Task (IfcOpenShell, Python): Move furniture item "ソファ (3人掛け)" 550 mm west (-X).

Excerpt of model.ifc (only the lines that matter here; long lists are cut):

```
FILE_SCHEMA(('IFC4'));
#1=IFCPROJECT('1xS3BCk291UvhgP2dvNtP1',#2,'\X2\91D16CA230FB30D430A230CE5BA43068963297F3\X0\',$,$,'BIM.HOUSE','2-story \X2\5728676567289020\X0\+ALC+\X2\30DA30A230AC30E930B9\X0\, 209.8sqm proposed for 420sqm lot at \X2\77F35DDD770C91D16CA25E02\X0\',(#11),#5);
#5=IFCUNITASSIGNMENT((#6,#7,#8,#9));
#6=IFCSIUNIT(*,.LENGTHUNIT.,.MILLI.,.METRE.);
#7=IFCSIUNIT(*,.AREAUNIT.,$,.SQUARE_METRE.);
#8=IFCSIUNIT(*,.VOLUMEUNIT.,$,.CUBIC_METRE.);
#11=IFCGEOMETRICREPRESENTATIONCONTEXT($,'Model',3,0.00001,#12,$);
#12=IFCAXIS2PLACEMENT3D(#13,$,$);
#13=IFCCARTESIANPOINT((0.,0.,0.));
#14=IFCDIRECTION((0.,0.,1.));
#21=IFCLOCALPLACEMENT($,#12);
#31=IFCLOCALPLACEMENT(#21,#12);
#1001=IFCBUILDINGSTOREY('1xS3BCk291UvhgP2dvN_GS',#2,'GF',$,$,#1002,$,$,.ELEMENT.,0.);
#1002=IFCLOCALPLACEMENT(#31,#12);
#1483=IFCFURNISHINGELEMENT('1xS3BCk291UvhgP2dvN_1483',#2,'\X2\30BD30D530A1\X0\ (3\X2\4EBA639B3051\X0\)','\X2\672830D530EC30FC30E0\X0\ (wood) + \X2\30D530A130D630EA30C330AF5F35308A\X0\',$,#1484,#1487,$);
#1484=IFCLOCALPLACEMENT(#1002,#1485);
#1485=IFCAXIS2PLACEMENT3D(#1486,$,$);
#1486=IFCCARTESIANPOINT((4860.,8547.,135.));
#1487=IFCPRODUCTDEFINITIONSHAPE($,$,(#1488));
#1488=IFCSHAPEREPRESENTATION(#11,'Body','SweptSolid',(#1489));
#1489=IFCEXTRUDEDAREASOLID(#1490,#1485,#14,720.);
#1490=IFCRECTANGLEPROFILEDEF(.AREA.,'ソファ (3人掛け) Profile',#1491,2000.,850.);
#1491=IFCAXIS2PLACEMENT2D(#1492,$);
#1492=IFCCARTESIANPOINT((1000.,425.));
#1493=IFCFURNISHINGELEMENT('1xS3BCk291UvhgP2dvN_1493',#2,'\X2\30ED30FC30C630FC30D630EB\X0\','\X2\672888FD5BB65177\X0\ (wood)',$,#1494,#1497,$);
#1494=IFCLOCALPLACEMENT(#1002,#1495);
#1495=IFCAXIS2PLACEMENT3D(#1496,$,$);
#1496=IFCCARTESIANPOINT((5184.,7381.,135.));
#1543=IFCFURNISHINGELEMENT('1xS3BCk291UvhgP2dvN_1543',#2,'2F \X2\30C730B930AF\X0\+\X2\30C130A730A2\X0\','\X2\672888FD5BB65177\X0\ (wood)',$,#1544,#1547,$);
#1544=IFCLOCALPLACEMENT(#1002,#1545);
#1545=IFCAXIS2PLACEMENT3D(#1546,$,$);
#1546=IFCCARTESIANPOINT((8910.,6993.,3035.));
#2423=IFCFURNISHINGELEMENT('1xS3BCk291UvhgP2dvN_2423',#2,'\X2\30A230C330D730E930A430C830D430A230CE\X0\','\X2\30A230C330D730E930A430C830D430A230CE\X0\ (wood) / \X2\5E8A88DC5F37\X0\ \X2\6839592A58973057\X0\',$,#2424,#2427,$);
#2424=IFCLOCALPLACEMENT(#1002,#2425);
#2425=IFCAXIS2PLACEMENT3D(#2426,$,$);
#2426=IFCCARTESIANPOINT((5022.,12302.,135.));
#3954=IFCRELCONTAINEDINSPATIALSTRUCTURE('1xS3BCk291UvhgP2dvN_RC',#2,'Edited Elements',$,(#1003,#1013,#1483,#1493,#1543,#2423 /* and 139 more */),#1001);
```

```python
import ifcopenshell
import ifcopenshell.api.geometry
import ifcopenshell.util.placement
import ifcopenshell.util.unit

model = ifcopenshell.open("model.ifc")
unit_scale = ifcopenshell.util.unit.calculate_unit_scale(model)

item = model.by_guid("1xS3BCk291UvhgP2dvN_1483")
matrix = ifcopenshell.util.placement.get_local_placement(item.ObjectPlacement)
matrix[0, 3] -= 0.55 / unit_scale
ifcopenshell.api.geometry.edit_object_placement(model, product=item, matrix=matrix, is_si=False)

print(ifcopenshell.util.placement.get_local_placement(item.ObjectPlacement).round(3) + 0.0)

model.write("model_updated.ifc")
```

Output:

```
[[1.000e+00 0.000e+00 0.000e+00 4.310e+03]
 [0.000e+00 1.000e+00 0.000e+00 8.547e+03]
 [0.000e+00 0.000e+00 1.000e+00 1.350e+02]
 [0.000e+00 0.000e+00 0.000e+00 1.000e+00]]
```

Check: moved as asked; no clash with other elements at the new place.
